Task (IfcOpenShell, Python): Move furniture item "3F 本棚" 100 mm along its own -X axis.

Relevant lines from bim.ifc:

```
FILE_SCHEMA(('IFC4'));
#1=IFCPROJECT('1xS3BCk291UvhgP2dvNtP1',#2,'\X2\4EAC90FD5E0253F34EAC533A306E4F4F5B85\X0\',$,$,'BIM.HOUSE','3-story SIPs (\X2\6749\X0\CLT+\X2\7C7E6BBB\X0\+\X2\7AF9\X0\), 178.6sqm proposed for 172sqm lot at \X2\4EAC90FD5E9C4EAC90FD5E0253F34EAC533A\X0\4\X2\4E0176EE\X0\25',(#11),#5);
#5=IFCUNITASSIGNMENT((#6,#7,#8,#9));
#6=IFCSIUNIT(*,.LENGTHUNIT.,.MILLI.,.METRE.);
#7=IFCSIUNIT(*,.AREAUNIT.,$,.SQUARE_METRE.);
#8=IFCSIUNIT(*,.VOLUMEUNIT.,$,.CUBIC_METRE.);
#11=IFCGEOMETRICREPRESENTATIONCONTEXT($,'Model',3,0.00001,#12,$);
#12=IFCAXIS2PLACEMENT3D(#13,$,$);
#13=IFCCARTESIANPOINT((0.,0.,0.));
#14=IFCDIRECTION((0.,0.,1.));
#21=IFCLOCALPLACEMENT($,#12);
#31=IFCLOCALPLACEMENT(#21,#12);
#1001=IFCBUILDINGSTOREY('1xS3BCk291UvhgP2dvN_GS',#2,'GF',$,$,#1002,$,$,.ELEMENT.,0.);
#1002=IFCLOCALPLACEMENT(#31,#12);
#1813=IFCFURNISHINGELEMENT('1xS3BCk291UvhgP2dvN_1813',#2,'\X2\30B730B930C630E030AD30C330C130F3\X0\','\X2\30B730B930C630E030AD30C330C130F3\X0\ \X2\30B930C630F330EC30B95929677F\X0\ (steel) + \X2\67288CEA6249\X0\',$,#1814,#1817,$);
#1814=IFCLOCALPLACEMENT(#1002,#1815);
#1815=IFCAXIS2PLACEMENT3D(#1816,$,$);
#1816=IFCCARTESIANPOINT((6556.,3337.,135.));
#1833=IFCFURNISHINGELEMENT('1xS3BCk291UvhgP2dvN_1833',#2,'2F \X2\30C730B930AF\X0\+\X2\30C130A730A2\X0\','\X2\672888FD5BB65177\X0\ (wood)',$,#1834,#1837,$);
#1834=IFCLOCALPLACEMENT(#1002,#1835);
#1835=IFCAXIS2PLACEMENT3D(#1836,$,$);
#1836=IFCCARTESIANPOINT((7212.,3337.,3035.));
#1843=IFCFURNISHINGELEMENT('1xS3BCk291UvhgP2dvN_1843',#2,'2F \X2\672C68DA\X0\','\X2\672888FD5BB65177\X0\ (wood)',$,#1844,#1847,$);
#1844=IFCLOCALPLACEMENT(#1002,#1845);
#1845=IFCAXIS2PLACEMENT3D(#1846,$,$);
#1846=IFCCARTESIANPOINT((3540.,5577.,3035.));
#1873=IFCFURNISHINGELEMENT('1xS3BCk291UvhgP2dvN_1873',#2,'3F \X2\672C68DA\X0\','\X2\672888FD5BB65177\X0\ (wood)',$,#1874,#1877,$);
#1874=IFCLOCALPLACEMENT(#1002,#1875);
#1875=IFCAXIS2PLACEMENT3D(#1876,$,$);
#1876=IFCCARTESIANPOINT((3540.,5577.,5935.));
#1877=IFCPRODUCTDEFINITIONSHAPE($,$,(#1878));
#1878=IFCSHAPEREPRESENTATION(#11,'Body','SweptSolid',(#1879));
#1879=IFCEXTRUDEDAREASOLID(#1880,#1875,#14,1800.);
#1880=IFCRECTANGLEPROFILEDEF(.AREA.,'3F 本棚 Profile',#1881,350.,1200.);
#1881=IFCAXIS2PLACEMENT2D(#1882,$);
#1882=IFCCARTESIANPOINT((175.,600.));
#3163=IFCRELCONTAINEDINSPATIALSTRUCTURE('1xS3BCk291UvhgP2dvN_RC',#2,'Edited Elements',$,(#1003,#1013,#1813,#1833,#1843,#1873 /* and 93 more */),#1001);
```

```python
import ifcopenshell
import ifcopenshell.api.geometry
import ifcopenshell.util.placement
import ifcopenshell.util.unit

model = ifcopenshell.open("bim.ifc")
unit_scale = ifcopenshell.util.unit.calculate_unit_scale(model)

item = model.by_guid("1xS3BCk291UvhgP2dvN_1873")
matrix = ifcopenshell.util.placement.get_local_placement(item.ObjectPlacement)
matrix[:3, 3] -= matrix[:3, 0] * 0.1 / unit_scale
ifcopenshell.api.geometry.edit_object_placement(model, product=item, matrix=matrix, is_si=False)

print(ifcopenshell.util.placement.get_local_placement(item.ObjectPlacement).round(3) + 0.0)

model.write("bim-out.ifc")
```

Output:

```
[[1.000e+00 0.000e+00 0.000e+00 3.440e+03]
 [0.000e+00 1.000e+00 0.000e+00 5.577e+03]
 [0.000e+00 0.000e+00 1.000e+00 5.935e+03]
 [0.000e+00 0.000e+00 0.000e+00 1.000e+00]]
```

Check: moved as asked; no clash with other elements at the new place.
